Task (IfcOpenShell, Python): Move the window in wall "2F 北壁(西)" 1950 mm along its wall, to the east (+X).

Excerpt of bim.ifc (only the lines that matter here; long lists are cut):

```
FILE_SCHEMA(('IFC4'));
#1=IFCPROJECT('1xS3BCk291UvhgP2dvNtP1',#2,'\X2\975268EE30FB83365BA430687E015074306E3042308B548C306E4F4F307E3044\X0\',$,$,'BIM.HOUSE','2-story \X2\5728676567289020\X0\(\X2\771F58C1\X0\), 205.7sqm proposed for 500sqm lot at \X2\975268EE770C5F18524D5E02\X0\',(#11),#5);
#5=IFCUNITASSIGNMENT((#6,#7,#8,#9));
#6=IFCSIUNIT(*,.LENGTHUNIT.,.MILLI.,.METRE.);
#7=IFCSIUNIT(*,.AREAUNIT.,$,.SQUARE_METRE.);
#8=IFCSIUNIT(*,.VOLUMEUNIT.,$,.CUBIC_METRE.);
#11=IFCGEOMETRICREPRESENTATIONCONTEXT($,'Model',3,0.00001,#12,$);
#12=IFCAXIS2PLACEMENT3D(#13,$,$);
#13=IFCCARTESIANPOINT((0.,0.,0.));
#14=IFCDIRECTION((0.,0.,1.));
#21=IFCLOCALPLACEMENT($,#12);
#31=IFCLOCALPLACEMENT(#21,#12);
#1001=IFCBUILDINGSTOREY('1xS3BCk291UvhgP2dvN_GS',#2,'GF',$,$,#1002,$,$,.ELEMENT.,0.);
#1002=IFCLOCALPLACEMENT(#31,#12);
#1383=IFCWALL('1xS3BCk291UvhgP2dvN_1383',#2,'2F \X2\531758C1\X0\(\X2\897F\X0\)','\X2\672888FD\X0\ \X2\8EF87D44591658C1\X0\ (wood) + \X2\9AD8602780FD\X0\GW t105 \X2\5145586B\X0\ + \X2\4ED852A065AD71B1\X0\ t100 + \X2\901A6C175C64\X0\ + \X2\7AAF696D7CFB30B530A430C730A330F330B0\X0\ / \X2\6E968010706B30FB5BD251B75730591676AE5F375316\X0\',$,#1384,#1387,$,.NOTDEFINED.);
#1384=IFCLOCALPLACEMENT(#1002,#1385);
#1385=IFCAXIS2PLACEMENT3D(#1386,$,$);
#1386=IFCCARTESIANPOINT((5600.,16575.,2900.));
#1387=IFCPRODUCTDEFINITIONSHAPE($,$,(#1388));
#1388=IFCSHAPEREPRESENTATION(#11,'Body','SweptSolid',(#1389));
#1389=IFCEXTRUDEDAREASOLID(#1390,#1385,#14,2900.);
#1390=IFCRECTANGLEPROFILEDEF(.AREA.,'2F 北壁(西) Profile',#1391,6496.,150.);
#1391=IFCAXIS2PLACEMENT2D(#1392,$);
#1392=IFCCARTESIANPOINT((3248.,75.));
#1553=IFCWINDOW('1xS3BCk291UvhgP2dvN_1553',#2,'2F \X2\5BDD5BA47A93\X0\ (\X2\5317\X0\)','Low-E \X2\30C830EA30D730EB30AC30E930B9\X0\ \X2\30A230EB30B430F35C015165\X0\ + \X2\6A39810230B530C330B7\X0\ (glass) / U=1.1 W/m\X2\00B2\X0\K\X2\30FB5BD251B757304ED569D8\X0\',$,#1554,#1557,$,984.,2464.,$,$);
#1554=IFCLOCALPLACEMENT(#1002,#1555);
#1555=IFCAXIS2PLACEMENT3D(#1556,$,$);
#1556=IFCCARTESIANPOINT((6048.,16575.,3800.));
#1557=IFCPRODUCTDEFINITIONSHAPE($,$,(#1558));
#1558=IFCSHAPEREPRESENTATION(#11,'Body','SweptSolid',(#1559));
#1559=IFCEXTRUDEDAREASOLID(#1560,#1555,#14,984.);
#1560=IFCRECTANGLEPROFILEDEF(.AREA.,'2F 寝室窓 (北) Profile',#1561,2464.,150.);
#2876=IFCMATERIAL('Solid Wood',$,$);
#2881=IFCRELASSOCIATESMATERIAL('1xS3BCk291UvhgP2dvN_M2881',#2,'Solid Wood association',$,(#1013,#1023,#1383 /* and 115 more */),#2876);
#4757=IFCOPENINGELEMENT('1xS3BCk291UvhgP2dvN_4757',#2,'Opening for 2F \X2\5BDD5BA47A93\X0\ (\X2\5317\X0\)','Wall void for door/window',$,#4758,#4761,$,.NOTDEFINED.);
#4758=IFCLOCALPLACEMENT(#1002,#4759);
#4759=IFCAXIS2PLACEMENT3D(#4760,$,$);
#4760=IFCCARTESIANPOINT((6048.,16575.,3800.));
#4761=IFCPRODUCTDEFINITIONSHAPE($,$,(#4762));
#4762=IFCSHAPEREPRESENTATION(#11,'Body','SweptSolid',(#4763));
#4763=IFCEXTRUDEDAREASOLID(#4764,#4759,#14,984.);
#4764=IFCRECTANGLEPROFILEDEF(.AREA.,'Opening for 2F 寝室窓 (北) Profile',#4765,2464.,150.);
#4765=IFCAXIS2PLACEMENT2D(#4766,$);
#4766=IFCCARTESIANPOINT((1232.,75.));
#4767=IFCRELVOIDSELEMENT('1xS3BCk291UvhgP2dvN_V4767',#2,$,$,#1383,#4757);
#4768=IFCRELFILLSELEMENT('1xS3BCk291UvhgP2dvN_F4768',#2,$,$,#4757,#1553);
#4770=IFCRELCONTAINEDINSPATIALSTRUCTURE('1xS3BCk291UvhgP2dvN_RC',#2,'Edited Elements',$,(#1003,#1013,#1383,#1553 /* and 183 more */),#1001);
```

```python
import ifcopenshell
import ifcopenshell.api.geometry
import ifcopenshell.util.placement

model = ifcopenshell.open("bim.ifc")

window = model.by_guid("1xS3BCk291UvhgP2dvN_1553")
opening = window.FillsVoids[0].RelatingOpeningElement
wall = opening.VoidsElements[0].RelatingBuildingElement

wall_matrix = ifcopenshell.util.placement.get_local_placement(wall.ObjectPlacement)
shift = wall_matrix[:3, 0] * 1950.0
before = ifcopenshell.util.placement.get_local_placement(window.ObjectPlacement)[:3, 3].copy()

# The window is not placed relative to its opening, so move both.
for product in (opening, window):
    matrix = ifcopenshell.util.placement.get_local_placement(product.ObjectPlacement)
    matrix[:3, 3] += shift
    ifcopenshell.api.geometry.edit_object_placement(model, product=product, matrix=matrix, is_si=False)

after = ifcopenshell.util.placement.get_local_placement(window.ObjectPlacement)[:3, 3]
print("window moved by", (after - before).round(3) + 0.0)

model.write("bim_v2.ifc")
```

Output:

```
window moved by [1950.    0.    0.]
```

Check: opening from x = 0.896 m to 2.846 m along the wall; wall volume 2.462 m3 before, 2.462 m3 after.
